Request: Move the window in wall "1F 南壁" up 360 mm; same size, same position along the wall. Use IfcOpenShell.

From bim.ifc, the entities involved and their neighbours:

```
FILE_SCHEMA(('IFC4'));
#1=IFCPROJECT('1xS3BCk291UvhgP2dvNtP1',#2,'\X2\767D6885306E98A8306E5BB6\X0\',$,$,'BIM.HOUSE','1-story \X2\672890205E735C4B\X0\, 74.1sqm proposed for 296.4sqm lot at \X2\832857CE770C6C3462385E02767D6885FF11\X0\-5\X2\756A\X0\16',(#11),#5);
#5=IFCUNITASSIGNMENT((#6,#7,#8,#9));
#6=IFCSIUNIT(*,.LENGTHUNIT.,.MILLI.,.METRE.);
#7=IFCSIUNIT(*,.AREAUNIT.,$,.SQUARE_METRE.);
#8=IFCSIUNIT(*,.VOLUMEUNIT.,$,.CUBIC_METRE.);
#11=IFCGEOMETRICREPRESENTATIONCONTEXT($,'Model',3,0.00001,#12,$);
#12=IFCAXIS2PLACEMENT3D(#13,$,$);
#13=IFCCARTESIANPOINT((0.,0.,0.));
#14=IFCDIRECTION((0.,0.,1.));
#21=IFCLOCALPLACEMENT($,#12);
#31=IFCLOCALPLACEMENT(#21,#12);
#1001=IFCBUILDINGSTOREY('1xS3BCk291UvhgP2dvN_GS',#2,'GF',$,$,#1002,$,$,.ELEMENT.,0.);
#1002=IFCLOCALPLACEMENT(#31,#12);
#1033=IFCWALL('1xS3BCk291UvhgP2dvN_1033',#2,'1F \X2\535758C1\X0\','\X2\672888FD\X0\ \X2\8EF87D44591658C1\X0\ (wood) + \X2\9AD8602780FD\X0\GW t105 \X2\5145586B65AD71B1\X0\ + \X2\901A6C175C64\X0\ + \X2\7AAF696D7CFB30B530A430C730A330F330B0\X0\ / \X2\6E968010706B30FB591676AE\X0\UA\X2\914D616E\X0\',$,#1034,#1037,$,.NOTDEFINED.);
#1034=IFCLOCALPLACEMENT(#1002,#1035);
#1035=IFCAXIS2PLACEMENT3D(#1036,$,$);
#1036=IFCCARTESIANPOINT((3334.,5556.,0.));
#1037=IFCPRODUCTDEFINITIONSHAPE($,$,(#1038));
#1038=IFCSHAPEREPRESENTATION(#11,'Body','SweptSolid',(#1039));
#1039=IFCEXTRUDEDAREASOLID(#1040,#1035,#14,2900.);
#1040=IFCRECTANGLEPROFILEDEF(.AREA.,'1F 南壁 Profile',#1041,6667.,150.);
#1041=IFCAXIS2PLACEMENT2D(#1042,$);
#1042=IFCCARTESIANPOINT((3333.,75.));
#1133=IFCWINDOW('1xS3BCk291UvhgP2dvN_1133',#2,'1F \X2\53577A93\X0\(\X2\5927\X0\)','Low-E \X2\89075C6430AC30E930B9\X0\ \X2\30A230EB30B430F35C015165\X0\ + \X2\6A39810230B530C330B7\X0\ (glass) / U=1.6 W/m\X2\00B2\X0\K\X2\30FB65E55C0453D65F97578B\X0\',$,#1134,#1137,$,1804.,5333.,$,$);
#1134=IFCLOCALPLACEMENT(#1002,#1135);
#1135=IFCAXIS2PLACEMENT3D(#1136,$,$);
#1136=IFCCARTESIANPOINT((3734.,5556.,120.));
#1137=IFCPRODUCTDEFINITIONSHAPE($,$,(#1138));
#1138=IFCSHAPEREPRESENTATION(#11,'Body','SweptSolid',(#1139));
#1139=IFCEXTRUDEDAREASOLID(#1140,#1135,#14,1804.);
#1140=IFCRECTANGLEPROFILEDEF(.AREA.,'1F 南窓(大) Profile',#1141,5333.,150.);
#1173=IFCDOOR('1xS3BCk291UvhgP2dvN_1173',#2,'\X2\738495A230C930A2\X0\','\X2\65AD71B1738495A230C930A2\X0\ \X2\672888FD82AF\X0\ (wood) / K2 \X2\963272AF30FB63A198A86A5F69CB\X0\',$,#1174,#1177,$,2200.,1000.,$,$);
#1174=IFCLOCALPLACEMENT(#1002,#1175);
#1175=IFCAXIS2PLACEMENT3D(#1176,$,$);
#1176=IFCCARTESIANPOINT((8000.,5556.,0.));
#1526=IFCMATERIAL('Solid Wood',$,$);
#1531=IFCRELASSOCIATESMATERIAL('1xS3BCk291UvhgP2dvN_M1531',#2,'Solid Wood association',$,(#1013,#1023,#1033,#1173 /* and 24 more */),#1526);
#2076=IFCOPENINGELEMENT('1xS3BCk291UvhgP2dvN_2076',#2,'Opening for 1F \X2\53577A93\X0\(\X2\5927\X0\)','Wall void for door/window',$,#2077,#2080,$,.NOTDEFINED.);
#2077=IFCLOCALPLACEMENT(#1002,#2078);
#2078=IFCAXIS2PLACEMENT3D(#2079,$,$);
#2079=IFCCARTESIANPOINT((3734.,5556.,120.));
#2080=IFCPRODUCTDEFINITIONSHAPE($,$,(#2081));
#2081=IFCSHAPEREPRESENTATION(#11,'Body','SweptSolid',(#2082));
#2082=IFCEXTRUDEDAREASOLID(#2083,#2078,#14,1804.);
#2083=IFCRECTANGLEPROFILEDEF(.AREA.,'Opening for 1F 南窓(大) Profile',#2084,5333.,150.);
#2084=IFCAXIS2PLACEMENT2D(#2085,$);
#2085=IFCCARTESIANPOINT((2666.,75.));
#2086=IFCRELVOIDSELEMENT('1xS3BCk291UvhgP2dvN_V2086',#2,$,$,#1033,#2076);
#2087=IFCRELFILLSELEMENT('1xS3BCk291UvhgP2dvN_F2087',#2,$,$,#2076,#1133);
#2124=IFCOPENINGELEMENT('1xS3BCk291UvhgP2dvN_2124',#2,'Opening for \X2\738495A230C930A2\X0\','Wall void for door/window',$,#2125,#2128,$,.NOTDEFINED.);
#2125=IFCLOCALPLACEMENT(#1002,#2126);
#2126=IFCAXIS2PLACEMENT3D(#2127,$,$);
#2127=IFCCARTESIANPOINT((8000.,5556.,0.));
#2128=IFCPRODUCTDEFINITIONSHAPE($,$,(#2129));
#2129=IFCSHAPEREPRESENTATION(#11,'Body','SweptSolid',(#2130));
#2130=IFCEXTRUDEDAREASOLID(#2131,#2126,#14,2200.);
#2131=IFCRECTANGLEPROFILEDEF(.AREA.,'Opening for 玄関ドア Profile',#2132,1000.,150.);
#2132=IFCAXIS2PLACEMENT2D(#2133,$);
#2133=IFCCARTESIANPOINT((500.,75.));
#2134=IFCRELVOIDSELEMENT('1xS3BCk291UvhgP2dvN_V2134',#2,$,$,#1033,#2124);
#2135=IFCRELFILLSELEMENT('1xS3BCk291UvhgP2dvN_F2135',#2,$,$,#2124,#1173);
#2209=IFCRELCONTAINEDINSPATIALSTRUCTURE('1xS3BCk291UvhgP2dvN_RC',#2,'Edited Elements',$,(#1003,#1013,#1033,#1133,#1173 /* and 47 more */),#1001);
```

```python
import numpy as np
import ifcopenshell
import ifcopenshell.api.geometry
import ifcopenshell.util.placement
import ifcopenshell.util.unit

model = ifcopenshell.open("bim.ifc")
unit_scale = ifcopenshell.util.unit.calculate_unit_scale(model)

window = model.by_guid("1xS3BCk291UvhgP2dvN_1133")
opening = window.FillsVoids[0].RelatingOpeningElement
dz = 0.36 / unit_scale

shift = np.array([0.0, 0.0, dz])
# The window is not placed relative to its opening, so move both.
for product in (opening, window):
    matrix = ifcopenshell.util.placement.get_local_placement(product.ObjectPlacement)
    matrix[:3, 3] += shift
    ifcopenshell.api.geometry.edit_object_placement(model, product=product, matrix=matrix, is_si=False)

print(f"moved by {dz * unit_scale:+.3f} m")

model.write("bim_updated.ifc")
```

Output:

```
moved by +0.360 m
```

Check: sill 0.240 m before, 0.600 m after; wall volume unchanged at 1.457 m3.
